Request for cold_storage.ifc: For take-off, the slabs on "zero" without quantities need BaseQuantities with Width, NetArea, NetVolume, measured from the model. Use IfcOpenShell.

First a look at what the model holds.

```python
import ifcopenshell
import ifcopenshell.util.element
import ifcopenshell.util.unit

model = ifcopenshell.open("cold_storage.ifc")
print(model.schema)
for unit_type in ("LENGTHUNIT", "AREAUNIT", "VOLUMEUNIT"):
    print(unit_type, ifcopenshell.util.unit.calculate_unit_scale(model, unit_type))
storey = next(s for s in model.by_type("IfcBuildingStorey") if s.Name == "zero")
slabs = [e for e in ifcopenshell.util.element.get_decomposition(storey) if e.is_a("IfcSlab")]
for e in sorted(slabs, key=lambda e: e.id()):
    print(e.id(), e.is_a(), e.Name, list(ifcopenshell.util.element.get_psets(e, qtos_only=True)), sep=" | ")
```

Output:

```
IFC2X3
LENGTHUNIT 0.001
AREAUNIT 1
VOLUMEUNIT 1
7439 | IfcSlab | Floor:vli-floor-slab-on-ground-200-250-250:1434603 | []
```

```python
import ifcopenshell
import ifcopenshell.api.pset
import ifcopenshell.geom
import ifcopenshell.util.element
import ifcopenshell.util.shape
import ifcopenshell.util.unit

model = ifcopenshell.open("cold_storage.ifc")
unit_scale = ifcopenshell.util.unit.calculate_unit_scale(model)
area_scale = ifcopenshell.util.unit.calculate_unit_scale(model, "AREAUNIT")
volume_scale = ifcopenshell.util.unit.calculate_unit_scale(model, "VOLUMEUNIT")
settings = ifcopenshell.geom.settings()

storey = next(s for s in model.by_type("IfcBuildingStorey") if s.Name == "zero")
slabs = [e for e in ifcopenshell.util.element.get_decomposition(storey) if e.is_a("IfcSlab")]

for e in sorted(slabs, key=lambda e: e.id()):
    if ifcopenshell.util.element.get_psets(e, qtos_only=True, should_inherit=False):
        continue
    # Geometry comes back in metres, in the element's own axes.
    shape = ifcopenshell.geom.create_shape(settings, e)
    values = {
        "Width": ifcopenshell.util.shape.get_z(shape.geometry) / unit_scale,
        "NetArea": ifcopenshell.util.shape.get_footprint_area(shape.geometry) / area_scale,
        "NetVolume": ifcopenshell.util.shape.get_volume(shape.geometry) / volume_scale,
    }
    qto = ifcopenshell.api.pset.add_qto(model, product=e, name="BaseQuantities")
    ifcopenshell.api.pset.edit_qto(model, qto=qto, properties=values)
    print(e.id(), {k: round(v, 3) for k, v in values.items()})

model.write("cold_storage_edited.ifc")
```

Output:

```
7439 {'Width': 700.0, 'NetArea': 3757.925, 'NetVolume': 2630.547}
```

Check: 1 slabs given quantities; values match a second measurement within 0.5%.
